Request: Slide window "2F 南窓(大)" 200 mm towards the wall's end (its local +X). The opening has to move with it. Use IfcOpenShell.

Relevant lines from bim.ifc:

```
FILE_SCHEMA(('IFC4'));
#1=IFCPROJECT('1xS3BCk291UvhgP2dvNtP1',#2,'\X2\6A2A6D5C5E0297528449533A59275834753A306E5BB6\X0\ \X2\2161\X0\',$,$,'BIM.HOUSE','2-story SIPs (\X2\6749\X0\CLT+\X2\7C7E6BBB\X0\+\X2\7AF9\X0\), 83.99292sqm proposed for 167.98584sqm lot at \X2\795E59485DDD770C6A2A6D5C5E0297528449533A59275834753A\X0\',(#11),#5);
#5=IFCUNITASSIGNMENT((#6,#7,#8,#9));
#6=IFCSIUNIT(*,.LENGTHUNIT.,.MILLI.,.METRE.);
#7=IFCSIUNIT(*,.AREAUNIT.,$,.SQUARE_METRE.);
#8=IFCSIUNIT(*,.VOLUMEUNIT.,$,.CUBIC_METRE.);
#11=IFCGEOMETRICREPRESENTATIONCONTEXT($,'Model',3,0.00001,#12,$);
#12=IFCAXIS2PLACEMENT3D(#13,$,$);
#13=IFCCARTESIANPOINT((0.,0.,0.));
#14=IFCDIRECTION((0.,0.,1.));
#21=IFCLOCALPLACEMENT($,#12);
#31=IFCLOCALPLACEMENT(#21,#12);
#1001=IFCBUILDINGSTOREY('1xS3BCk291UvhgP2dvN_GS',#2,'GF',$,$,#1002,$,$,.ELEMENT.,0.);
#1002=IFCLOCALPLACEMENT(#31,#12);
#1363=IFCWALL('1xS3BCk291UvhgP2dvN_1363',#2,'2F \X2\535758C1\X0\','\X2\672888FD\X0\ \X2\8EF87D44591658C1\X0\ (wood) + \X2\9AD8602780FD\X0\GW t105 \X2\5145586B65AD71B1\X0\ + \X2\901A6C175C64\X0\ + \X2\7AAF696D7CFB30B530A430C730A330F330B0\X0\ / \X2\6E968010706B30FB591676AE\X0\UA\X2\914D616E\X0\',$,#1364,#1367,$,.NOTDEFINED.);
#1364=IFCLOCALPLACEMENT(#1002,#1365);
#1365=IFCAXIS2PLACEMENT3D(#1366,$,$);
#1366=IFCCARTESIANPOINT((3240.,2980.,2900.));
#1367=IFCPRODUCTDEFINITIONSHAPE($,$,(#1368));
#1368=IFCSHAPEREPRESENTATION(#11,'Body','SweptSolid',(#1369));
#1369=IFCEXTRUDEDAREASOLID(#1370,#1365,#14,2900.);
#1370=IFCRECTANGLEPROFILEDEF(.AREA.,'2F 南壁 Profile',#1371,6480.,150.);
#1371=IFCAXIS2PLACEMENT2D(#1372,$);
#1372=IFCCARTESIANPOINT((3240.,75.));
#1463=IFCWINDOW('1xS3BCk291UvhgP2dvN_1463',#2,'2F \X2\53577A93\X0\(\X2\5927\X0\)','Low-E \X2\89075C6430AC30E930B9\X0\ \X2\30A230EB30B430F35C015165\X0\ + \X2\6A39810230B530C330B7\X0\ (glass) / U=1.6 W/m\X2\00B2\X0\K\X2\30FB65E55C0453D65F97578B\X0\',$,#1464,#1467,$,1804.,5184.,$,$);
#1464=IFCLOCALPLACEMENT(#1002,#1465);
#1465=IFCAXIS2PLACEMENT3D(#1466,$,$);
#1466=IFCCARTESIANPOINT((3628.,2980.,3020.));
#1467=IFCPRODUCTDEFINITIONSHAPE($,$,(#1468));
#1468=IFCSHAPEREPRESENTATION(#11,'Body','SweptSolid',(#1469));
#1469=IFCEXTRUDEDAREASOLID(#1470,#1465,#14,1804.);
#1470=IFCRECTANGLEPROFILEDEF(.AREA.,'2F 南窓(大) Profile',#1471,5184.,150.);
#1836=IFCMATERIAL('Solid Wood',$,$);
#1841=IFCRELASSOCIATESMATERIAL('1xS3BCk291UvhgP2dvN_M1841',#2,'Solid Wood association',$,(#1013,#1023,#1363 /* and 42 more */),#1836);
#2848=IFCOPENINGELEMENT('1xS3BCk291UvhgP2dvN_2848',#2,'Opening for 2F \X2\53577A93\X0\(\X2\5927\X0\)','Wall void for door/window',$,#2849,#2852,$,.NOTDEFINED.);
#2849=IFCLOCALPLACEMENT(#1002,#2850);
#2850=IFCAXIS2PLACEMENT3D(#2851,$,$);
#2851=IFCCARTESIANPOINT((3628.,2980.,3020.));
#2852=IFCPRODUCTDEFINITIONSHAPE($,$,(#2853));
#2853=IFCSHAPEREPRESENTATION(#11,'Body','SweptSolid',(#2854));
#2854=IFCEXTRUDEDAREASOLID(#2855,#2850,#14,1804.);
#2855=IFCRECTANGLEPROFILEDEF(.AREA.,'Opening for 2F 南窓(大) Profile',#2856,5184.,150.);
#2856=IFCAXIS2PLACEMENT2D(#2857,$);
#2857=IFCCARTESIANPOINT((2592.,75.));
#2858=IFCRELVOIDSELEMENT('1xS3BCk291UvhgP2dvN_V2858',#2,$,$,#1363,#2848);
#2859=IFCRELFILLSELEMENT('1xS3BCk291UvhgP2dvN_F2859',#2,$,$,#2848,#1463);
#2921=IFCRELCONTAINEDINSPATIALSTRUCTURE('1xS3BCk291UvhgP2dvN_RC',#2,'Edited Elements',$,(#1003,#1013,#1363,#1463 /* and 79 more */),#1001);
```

```python
import ifcopenshell
import ifcopenshell.api.geometry
import ifcopenshell.util.placement
import ifcopenshell.util.unit

model = ifcopenshell.open("bim.ifc")
unit_scale = ifcopenshell.util.unit.calculate_unit_scale(model)

window = model.by_id(1463)
opening = window.FillsVoids[0].RelatingOpeningElement
wall = opening.VoidsElements[0].RelatingBuildingElement

wall_matrix = ifcopenshell.util.placement.get_local_placement(wall.ObjectPlacement)
shift = wall_matrix[:3, 0] * 0.2 / unit_scale
before = ifcopenshell.util.placement.get_local_placement(window.ObjectPlacement)[:3, 3].copy()

# The window is not placed relative to its opening, so move both.
for product in (opening, window):
    matrix = ifcopenshell.util.placement.get_local_placement(product.ObjectPlacement)
    matrix[:3, 3] += shift
    ifcopenshell.api.geometry.edit_object_placement(model, product=product, matrix=matrix, is_si=False)

after = ifcopenshell.util.placement.get_local_placement(window.ObjectPlacement)[:3, 3]
print("window moved by", (after - before).round(3) + 0.0)

model.write("bim_edited.ifc")
```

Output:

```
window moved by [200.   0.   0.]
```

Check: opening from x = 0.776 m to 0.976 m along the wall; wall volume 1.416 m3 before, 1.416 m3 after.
